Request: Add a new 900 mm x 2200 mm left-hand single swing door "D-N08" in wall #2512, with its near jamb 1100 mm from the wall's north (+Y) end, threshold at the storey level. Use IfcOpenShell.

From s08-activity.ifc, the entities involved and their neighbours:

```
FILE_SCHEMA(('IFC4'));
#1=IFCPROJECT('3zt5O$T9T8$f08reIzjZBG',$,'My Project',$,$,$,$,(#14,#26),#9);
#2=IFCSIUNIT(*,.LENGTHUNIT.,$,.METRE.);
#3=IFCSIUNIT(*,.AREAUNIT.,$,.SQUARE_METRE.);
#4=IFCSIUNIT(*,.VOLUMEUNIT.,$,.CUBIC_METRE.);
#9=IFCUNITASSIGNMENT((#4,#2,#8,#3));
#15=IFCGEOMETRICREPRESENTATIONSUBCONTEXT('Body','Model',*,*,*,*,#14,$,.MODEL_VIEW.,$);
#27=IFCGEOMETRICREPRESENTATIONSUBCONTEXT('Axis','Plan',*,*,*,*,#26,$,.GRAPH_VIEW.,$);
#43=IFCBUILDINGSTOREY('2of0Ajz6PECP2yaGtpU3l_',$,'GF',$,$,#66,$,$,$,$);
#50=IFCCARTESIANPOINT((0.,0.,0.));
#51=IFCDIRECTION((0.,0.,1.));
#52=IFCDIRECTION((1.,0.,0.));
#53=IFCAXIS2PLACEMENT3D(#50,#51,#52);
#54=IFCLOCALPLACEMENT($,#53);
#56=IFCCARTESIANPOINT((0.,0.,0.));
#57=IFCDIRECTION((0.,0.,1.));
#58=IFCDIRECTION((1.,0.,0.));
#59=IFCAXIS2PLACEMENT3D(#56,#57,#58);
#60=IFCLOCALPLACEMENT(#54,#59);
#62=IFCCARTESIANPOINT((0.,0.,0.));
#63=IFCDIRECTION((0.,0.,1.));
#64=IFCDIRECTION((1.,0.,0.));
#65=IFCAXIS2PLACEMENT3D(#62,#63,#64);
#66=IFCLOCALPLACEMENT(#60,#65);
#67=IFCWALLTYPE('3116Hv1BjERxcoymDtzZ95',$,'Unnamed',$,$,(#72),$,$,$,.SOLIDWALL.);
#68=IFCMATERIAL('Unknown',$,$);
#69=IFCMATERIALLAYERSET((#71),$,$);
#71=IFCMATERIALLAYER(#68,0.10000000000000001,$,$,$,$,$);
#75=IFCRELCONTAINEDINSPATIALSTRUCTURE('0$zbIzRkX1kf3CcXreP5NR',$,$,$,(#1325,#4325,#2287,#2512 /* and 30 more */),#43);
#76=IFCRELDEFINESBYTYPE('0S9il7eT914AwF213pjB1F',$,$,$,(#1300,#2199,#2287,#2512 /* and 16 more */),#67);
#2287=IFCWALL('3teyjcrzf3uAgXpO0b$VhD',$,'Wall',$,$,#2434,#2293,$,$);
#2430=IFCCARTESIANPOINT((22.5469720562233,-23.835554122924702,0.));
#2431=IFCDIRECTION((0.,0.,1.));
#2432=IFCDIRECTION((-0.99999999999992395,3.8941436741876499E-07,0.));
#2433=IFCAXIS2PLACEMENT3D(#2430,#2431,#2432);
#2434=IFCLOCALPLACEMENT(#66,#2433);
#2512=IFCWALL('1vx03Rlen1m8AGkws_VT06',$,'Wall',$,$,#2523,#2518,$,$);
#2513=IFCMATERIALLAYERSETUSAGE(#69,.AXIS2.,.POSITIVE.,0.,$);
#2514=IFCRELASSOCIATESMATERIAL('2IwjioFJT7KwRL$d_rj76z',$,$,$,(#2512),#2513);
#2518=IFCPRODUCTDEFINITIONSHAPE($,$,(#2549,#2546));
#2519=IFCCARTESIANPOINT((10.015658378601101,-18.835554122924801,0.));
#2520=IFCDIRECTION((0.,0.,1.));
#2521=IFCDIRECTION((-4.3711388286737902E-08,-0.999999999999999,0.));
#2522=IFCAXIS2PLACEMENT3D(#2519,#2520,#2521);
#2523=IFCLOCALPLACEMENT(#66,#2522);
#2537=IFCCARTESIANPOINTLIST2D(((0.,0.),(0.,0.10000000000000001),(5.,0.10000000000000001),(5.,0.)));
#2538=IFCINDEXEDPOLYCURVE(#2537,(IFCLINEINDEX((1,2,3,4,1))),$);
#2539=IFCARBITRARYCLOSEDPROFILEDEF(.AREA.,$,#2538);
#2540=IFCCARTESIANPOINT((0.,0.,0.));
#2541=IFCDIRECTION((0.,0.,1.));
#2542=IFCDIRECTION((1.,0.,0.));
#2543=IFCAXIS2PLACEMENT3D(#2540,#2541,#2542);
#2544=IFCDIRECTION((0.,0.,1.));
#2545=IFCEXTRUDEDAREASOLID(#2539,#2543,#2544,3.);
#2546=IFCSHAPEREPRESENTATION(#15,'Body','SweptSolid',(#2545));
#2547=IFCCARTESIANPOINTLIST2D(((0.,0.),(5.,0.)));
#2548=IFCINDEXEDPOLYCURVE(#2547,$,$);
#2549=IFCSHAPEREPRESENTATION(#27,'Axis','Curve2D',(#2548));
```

```python
import numpy as np
import ifcopenshell
import ifcopenshell.api.feature
import ifcopenshell.api.geometry
import ifcopenshell.api.root
import ifcopenshell.api.spatial
import ifcopenshell.geom
import ifcopenshell.util.element
import ifcopenshell.util.placement
import ifcopenshell.util.representation
import ifcopenshell.util.shape
import ifcopenshell.util.unit

model = ifcopenshell.open("s08-activity.ifc")
unit_scale = ifcopenshell.util.unit.calculate_unit_scale(model)
settings = ifcopenshell.geom.settings()


def volume(element):
    """Net volume in cubic metres, openings subtracted."""
    shape = ifcopenshell.geom.create_shape(settings, element)
    return ifcopenshell.util.shape.get_volume(shape.geometry)


wall = model.by_guid("1vx03Rlen1m8AGkws_VT06")
storey = ifcopenshell.util.element.get_container(wall, ifc_class="IfcBuildingStorey")
context = ifcopenshell.util.representation.get_context(model, "Model", "Body", "MODEL_VIEW")
before = volume(wall)

width, height, from_end, sill = 0.9, 2.2, 1.1, 0.0  # metres

# The wall runs along its own X axis, and the end named is its -X end.
wall_shape = ifcopenshell.geom.create_shape(settings, wall)
x, y, z = ifcopenshell.util.shape.get_vertices(wall_shape.geometry).T
start = x.min() + from_end
face, thickness = float(y.min()), float(y.max() - y.min())
wall_matrix = ifcopenshell.util.placement.get_local_placement(wall.ObjectPlacement)
level = ifcopenshell.util.placement.get_local_placement(storey.ObjectPlacement)[2, 3]


def in_wall(x, y):
    """Placement at x, y metres in the wall's axes, at sill height."""
    matrix = wall_matrix.copy()
    matrix[:, 3] = wall_matrix @ np.array([x / unit_scale, y / unit_scale, 0.0, 1.0])
    matrix[2, 3] = level + sill / unit_scale
    return matrix


# Opening: a box that overshoots both wall faces by 50 mm.
opening = ifcopenshell.api.root.create_entity(model, ifc_class="IfcOpeningElement", predefined_type="OPENING")
box = ifcopenshell.api.geometry.add_wall_representation(
    model, context=context, length=width, height=height, thickness=thickness + 0.1
)
ifcopenshell.api.geometry.assign_representation(model, product=opening, representation=box)
ifcopenshell.api.geometry.edit_object_placement(model, product=opening, matrix=in_wall(start, face - 0.05), is_si=False)
ifcopenshell.api.feature.add_feature(model, feature=opening, element=wall)

door = ifcopenshell.api.root.create_entity(model, ifc_class="IfcDoor", name="D-N08", predefined_type="DOOR")
door.OverallWidth, door.OverallHeight = width / unit_scale, height / unit_scale
door.OperationType = "SINGLE_SWING_LEFT"
body = ifcopenshell.api.geometry.add_door_representation(
    model,
    context=context,
    overall_width=door.OverallWidth,
    overall_height=door.OverallHeight,
    operation_type="SINGLE_SWING_LEFT",
    lining_properties={"LiningDepth": thickness / unit_scale, "ThresholdDepth": thickness / unit_scale},
)
ifcopenshell.api.geometry.assign_representation(model, product=door, representation=body)
ifcopenshell.api.spatial.assign_container(model, products=[door], relating_structure=storey)
ifcopenshell.api.feature.add_filling(model, opening=opening, element=door)

# The lining spans the wall, so the door starts at the wall face.
ifcopenshell.api.geometry.edit_object_placement(model, product=door, matrix=in_wall(start, face), is_si=False)

after = volume(wall)

print(f"wall volume {before:.3f} -> {after:.3f} m3")

model.write("s08-activity_updated.ifc")
```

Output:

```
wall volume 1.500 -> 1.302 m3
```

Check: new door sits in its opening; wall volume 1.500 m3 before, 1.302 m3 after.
